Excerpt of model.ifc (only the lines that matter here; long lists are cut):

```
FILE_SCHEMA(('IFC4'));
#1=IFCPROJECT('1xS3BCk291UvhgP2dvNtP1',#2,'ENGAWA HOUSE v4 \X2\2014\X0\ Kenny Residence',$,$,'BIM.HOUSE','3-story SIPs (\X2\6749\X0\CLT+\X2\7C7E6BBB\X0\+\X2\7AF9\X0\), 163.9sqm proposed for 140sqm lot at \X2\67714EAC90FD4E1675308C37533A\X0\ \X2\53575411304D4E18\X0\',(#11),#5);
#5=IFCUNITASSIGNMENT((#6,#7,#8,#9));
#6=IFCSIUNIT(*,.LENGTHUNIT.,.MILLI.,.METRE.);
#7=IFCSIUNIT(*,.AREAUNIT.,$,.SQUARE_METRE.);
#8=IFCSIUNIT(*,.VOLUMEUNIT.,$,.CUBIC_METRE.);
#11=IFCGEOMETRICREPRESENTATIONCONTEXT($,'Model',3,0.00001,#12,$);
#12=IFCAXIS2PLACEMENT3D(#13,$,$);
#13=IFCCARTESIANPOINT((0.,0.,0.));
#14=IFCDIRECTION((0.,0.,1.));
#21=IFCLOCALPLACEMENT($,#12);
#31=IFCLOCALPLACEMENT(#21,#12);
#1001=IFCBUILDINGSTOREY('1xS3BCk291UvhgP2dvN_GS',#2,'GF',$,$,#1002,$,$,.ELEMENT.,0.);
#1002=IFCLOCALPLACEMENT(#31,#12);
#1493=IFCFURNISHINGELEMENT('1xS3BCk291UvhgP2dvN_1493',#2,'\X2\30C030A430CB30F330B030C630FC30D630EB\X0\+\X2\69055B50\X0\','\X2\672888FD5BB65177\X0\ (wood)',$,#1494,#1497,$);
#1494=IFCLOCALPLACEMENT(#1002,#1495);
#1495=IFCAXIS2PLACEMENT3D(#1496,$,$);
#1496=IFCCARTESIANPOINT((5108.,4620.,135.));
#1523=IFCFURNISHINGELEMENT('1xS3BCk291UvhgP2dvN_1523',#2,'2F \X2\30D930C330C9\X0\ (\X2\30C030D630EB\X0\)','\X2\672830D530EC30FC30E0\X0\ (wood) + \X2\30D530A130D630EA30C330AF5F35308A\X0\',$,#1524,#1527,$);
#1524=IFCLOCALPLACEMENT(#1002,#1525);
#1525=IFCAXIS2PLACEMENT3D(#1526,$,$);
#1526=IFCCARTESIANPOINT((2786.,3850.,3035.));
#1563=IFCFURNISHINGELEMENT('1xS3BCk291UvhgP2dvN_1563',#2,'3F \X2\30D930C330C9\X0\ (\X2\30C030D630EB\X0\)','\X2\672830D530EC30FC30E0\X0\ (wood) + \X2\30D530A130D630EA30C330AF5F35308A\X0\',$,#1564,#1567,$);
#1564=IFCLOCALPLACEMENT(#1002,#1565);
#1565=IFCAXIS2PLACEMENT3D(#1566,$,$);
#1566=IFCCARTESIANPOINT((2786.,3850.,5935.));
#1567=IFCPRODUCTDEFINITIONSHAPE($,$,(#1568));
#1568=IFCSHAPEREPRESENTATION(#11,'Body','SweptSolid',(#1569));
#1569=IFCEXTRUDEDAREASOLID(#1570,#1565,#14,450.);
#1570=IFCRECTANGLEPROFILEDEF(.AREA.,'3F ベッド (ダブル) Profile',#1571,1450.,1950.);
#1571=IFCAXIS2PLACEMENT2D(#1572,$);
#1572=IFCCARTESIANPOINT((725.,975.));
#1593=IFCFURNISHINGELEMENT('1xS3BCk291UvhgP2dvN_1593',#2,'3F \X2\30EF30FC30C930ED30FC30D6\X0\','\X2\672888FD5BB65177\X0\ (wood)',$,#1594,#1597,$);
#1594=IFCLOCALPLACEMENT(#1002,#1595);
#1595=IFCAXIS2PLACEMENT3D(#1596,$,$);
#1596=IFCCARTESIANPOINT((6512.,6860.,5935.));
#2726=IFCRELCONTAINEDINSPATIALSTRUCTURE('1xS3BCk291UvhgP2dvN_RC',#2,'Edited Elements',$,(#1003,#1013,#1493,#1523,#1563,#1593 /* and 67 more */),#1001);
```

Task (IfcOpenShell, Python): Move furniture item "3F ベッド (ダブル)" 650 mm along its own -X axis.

```python
import ifcopenshell
import ifcopenshell.api.geometry
import ifcopenshell.util.placement
import ifcopenshell.util.unit

model = ifcopenshell.open("model.ifc")
unit_scale = ifcopenshell.util.unit.calculate_unit_scale(model)

item = model.by_id(1563)
matrix = ifcopenshell.util.placement.get_local_placement(item.ObjectPlacement)
matrix[:3, 3] -= matrix[:3, 0] * 0.65 / unit_scale
ifcopenshell.api.geometry.edit_object_placement(model, product=item, matrix=matrix, is_si=False)

print(ifcopenshell.util.placement.get_local_placement(item.ObjectPlacement).round(3) + 0.0)

model.write("model-out.ifc")
```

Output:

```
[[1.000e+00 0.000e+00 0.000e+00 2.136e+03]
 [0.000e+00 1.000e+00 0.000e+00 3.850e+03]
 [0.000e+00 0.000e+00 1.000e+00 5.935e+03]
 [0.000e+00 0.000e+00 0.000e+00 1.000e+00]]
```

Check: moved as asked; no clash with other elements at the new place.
